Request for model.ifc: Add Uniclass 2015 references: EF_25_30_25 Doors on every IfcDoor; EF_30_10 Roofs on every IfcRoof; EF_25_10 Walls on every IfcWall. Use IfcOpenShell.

First a look at what the model holds.

```python
import ifcopenshell

model = ifcopenshell.open("model.ifc")
print(model.schema)
print("classifications:", [c.Name for c in model.by_type("IfcClassification")])
for ifc_class in ("IfcDoor", "IfcRoof", "IfcStair", "IfcWall", "IfcWindow"):
    print(ifc_class, len(model.by_type(ifc_class)))
```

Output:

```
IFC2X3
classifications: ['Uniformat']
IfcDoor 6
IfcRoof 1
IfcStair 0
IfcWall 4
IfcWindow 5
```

```python
import ifcopenshell
import ifcopenshell.api.classification

model = ifcopenshell.open("model.ifc")

# IFC2X3 requires Source and Edition and has no link from the project to the system.
system = model.create_entity("IfcClassification", Source="NBS", Edition="2015", Name="Uniclass 2015")

codes = {
    "IfcDoor": ("EF_25_30_25", "Doors"),
    "IfcRoof": ("EF_30_10", "Roofs"),
    "IfcWall": ("EF_25_10", "Walls"),
}
for ifc_class, (code, name) in codes.items():
    products = model.by_type(ifc_class)
    ifcopenshell.api.classification.add_reference(
        model, products=products, classification=system, identification=code, name=name
    )
    print(code, len(products))

model.write("model-out.ifc")
```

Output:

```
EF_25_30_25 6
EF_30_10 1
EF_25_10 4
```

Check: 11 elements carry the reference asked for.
